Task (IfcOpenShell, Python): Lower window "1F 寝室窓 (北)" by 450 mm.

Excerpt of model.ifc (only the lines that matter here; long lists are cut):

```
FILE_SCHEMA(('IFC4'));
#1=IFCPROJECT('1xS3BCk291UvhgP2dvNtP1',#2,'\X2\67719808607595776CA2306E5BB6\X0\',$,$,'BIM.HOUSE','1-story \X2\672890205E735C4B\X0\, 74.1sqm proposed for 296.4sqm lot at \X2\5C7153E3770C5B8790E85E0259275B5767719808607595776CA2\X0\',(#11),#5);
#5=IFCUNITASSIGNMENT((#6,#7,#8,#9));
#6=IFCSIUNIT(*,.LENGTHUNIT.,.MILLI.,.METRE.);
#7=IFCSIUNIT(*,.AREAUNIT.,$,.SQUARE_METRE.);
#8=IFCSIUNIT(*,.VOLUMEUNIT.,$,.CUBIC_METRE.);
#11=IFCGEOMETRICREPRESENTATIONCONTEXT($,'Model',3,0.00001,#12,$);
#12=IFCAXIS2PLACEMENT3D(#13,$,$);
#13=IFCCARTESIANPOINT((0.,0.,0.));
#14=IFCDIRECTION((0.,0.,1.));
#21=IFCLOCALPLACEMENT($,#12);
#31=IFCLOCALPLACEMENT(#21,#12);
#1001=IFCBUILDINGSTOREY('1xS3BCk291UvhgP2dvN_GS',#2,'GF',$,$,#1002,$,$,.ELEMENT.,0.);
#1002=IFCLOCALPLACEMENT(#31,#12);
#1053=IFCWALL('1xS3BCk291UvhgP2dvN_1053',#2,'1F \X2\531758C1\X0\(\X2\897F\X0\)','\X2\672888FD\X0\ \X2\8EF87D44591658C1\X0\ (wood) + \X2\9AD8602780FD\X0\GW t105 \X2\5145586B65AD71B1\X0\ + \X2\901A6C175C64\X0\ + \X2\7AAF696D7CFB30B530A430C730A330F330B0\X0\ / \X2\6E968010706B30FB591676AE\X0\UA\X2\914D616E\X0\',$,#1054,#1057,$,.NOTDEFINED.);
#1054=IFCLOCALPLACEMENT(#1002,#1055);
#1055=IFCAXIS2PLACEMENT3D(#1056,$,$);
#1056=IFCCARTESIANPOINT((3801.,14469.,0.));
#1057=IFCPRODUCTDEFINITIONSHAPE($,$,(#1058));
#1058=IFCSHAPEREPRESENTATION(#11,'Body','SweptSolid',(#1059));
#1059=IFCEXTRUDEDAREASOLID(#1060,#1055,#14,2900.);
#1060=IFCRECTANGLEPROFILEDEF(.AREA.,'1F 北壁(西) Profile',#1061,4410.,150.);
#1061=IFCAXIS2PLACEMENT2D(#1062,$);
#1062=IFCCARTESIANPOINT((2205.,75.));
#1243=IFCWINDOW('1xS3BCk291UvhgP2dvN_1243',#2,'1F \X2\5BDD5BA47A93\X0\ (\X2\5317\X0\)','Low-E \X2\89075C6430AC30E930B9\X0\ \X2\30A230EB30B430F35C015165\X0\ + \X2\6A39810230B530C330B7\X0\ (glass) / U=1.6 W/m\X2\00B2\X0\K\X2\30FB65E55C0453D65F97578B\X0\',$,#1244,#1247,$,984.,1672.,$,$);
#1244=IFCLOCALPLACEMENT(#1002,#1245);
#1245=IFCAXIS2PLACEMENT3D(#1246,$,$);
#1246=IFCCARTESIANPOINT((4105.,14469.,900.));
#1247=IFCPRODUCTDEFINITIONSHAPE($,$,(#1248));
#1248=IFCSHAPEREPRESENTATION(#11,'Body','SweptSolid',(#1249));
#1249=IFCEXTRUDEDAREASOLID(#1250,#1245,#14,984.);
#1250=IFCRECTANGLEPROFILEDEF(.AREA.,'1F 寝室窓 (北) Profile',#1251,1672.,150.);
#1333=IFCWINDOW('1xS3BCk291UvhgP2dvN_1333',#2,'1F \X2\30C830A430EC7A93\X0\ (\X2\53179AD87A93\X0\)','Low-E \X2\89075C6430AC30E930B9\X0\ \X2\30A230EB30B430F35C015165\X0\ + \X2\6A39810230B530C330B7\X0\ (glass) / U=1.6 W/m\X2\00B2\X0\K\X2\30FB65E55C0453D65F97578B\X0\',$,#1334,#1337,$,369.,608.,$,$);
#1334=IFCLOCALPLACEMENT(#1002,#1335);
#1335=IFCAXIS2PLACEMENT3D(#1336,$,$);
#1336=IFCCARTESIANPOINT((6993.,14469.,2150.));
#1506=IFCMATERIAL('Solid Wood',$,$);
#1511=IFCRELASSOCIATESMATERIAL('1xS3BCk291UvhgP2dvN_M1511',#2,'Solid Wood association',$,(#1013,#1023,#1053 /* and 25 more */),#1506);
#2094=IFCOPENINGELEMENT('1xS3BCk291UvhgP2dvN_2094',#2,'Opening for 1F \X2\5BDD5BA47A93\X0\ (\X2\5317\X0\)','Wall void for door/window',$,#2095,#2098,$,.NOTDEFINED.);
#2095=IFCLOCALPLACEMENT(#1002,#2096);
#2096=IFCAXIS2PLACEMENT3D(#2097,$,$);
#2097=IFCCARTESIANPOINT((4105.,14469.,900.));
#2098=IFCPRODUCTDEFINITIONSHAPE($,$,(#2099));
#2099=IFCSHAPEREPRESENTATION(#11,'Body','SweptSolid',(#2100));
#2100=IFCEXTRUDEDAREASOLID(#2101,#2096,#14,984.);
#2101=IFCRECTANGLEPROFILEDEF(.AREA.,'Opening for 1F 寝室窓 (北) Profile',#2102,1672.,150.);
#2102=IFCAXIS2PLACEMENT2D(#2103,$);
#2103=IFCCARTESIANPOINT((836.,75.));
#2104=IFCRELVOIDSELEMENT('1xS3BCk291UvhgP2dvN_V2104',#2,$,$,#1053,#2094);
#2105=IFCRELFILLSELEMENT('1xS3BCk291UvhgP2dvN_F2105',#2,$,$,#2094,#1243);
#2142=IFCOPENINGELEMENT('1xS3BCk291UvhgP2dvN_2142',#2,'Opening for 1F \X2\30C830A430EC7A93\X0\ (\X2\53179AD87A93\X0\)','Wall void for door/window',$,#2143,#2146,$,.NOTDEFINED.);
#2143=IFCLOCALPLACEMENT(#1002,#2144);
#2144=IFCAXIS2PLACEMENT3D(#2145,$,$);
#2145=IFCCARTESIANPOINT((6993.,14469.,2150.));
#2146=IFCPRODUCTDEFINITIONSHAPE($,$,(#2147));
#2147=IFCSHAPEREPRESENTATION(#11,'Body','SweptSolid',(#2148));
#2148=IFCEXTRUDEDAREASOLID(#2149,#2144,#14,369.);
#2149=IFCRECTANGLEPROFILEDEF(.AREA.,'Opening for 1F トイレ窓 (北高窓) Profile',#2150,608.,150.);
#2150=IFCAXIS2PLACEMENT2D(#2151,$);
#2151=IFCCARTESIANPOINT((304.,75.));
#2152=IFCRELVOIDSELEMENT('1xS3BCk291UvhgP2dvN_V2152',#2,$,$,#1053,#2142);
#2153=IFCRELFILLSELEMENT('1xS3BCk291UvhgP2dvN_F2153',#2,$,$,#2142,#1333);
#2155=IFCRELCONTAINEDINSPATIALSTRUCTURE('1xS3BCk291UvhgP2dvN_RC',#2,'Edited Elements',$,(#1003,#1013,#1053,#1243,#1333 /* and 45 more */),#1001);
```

```python
import numpy as np
import ifcopenshell
import ifcopenshell.api.geometry
import ifcopenshell.util.placement
import ifcopenshell.util.unit

model = ifcopenshell.open("model.ifc")
unit_scale = ifcopenshell.util.unit.calculate_unit_scale(model)

window = model.by_id(1243)
opening = window.FillsVoids[0].RelatingOpeningElement
dz = -450.0

shift = np.array([0.0, 0.0, dz])
# The window is not placed relative to its opening, so move both.
for product in (opening, window):
    matrix = ifcopenshell.util.placement.get_local_placement(product.ObjectPlacement)
    matrix[:3, 3] += shift
    ifcopenshell.api.geometry.edit_object_placement(model, product=product, matrix=matrix, is_si=False)

print(f"moved by {dz * unit_scale:+.3f} m")

model.write("model_updated.ifc")
```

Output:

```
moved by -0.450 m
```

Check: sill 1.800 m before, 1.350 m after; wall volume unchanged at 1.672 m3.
